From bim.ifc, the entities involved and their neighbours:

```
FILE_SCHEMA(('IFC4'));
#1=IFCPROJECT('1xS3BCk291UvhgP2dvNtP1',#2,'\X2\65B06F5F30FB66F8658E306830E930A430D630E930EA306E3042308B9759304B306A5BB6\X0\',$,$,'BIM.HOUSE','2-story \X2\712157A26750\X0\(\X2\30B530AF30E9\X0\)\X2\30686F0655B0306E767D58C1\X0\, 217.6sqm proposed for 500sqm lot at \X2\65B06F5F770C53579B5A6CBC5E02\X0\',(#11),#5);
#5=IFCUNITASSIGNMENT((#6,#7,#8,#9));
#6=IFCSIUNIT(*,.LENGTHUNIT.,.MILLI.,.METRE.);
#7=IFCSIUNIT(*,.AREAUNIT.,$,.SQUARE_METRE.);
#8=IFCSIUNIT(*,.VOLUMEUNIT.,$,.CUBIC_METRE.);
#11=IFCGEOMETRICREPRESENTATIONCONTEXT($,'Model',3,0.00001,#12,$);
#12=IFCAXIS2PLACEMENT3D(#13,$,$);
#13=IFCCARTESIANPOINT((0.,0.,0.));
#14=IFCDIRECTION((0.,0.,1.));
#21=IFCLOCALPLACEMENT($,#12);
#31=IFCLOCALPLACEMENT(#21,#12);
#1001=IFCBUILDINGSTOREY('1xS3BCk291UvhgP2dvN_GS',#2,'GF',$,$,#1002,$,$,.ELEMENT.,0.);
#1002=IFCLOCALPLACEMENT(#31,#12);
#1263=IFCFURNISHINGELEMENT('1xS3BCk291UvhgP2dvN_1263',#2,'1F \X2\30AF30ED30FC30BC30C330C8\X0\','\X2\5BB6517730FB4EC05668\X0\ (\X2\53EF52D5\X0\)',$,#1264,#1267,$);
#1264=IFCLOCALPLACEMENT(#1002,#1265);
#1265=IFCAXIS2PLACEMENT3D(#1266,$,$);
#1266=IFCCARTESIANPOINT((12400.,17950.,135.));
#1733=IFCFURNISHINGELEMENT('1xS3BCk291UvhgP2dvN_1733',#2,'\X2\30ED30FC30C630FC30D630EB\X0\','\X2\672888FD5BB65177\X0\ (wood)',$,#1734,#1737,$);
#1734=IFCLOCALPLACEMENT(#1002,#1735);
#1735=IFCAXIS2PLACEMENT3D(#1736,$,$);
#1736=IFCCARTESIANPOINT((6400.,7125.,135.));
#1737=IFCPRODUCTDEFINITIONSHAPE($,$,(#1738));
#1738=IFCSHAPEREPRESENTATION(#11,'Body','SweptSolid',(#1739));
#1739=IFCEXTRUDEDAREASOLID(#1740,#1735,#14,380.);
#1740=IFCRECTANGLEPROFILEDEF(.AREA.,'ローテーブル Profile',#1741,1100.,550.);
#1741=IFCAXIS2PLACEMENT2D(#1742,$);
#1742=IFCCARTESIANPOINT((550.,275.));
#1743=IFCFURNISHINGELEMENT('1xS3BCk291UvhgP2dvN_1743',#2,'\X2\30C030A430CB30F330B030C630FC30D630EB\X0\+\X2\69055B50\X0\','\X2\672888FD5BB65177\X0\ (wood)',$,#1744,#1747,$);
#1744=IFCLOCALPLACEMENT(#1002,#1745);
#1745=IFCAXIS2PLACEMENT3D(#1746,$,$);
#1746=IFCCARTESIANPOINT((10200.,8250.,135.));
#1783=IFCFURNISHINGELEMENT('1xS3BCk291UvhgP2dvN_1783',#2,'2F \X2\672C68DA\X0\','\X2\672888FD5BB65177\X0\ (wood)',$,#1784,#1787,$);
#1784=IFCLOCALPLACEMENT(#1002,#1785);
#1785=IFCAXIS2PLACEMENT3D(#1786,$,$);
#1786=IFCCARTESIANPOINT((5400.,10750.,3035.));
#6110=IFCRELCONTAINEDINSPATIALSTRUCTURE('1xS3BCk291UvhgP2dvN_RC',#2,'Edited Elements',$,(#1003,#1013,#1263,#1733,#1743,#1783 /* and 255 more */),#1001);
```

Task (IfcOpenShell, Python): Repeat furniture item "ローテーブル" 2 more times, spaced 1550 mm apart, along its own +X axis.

```python
import ifcopenshell
import ifcopenshell.api.geometry
import ifcopenshell.api.root
import ifcopenshell.util.element
import ifcopenshell.util.placement
import ifcopenshell.util.unit

model = ifcopenshell.open("bim.ifc")
unit_scale = ifcopenshell.util.unit.calculate_unit_scale(model)


def reuse_history(source, copy):
    """copy_class also copies each property set's owner history, people and application; keep the originals."""
    for rel in copy.IsDefinedBy:
        if rel.is_a("IfcRelDefinesByProperties") and (history := rel.RelatingPropertyDefinition.OwnerHistory):
            rel.RelatingPropertyDefinition.OwnerHistory = source.OwnerHistory
            ifcopenshell.util.element.remove_deep2(model, history)


source = model.by_guid("1xS3BCk291UvhgP2dvN_1733")
base = ifcopenshell.util.placement.get_local_placement(source.ObjectPlacement)
step = base[:3, 0] * 1.55 / unit_scale

for i in range(1, 3):
    copy = ifcopenshell.api.root.copy_class(model, product=source)
    copy.Representation = ifcopenshell.util.element.copy_deep(
        model, source.Representation, exclude=["IfcGeometricRepresentationContext", "IfcRepresentationMap"]
    )
    reuse_history(source, copy)
    matrix = base.copy()
    matrix[:3, 3] += i * step
    print("added at", matrix[:3, 3].round(3) + 0.0)
    ifcopenshell.api.geometry.edit_object_placement(model, product=copy, matrix=matrix, is_si=False)

model.write("bim_v2.ifc")
```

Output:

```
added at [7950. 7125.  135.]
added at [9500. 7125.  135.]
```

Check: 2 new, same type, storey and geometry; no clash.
